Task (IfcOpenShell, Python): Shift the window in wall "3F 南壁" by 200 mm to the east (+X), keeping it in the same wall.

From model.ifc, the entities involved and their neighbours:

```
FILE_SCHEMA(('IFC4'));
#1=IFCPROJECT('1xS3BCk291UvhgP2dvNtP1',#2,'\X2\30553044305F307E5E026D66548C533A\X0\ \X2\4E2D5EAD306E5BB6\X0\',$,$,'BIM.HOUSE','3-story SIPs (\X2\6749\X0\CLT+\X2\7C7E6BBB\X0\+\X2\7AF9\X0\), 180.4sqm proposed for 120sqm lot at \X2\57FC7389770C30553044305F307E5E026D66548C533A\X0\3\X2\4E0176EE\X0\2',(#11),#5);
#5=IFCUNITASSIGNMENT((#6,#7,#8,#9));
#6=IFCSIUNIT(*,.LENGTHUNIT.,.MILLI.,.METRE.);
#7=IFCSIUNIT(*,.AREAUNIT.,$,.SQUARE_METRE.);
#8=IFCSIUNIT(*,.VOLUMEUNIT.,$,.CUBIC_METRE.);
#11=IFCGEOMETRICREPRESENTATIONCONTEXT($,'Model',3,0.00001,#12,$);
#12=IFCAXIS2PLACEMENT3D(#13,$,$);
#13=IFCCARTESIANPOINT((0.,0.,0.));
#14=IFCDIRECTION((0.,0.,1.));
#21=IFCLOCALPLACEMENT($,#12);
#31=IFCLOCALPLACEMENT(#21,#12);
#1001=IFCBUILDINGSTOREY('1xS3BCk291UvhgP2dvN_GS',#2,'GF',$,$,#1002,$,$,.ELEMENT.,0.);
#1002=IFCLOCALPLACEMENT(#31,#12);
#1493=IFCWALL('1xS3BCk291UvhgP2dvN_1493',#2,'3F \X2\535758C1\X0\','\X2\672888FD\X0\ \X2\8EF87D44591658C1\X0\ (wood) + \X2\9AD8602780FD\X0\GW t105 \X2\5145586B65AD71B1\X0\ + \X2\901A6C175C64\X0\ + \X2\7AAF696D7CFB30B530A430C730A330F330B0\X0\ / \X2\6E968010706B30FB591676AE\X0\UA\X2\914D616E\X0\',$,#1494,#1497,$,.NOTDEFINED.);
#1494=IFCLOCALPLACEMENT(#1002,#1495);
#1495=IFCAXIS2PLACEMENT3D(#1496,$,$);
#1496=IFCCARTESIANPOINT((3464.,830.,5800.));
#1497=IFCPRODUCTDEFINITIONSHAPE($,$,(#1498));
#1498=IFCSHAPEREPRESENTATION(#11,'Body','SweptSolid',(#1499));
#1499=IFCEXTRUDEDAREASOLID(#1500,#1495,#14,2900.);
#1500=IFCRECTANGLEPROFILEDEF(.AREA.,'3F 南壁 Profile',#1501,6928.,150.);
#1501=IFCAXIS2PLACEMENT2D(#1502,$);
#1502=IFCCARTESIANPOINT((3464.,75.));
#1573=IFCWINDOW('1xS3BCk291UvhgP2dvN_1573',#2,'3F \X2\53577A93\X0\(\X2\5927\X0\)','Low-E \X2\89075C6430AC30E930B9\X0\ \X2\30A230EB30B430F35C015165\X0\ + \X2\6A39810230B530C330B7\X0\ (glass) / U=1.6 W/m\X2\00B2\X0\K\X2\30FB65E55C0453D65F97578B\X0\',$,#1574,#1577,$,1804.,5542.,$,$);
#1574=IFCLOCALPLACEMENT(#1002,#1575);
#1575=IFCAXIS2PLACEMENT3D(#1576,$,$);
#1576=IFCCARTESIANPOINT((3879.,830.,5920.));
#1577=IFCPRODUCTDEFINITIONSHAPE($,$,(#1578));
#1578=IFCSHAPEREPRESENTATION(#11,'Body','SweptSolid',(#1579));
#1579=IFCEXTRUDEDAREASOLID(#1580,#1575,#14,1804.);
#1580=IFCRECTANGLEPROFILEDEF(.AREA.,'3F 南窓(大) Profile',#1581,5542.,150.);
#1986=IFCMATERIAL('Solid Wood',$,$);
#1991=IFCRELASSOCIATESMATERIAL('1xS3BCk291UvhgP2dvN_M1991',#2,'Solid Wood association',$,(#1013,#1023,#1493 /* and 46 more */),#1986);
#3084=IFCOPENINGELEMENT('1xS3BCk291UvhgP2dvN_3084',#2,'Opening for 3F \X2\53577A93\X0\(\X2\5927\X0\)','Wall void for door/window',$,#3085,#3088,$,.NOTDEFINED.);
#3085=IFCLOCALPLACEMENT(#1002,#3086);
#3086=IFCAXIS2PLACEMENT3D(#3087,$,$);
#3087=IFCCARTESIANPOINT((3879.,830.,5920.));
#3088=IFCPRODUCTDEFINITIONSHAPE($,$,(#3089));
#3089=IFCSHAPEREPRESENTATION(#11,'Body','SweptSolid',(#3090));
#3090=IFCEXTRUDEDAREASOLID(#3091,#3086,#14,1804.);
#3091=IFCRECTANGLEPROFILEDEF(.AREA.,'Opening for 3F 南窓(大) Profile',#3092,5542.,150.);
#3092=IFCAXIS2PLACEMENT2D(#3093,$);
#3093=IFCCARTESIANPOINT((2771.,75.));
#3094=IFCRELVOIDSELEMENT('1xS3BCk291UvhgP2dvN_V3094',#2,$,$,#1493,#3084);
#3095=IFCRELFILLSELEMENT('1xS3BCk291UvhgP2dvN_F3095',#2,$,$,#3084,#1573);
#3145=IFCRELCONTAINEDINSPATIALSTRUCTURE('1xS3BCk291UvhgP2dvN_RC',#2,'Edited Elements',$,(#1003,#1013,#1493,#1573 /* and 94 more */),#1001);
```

```python
import ifcopenshell
import ifcopenshell.api.geometry
import ifcopenshell.util.placement
import ifcopenshell.util.unit

model = ifcopenshell.open("model.ifc")
unit_scale = ifcopenshell.util.unit.calculate_unit_scale(model)

window = model.by_guid("1xS3BCk291UvhgP2dvN_1573")
opening = window.FillsVoids[0].RelatingOpeningElement
wall = opening.VoidsElements[0].RelatingBuildingElement

wall_matrix = ifcopenshell.util.placement.get_local_placement(wall.ObjectPlacement)
shift = wall_matrix[:3, 0] * 0.2 / unit_scale
before = ifcopenshell.util.placement.get_local_placement(window.ObjectPlacement)[:3, 3].copy()

# The window is not placed relative to its opening, so move both.
for product in (opening, window):
    matrix = ifcopenshell.util.placement.get_local_placement(product.ObjectPlacement)
    matrix[:3, 3] += shift
    ifcopenshell.api.geometry.edit_object_placement(model, product=product, matrix=matrix, is_si=False)

after = ifcopenshell.util.placement.get_local_placement(window.ObjectPlacement)[:3, 3]
print("window moved by", (after - before).round(3) + 0.0)

model.write("model_edited.ifc")
```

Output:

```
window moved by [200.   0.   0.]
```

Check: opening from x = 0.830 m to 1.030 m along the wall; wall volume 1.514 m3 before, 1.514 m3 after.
